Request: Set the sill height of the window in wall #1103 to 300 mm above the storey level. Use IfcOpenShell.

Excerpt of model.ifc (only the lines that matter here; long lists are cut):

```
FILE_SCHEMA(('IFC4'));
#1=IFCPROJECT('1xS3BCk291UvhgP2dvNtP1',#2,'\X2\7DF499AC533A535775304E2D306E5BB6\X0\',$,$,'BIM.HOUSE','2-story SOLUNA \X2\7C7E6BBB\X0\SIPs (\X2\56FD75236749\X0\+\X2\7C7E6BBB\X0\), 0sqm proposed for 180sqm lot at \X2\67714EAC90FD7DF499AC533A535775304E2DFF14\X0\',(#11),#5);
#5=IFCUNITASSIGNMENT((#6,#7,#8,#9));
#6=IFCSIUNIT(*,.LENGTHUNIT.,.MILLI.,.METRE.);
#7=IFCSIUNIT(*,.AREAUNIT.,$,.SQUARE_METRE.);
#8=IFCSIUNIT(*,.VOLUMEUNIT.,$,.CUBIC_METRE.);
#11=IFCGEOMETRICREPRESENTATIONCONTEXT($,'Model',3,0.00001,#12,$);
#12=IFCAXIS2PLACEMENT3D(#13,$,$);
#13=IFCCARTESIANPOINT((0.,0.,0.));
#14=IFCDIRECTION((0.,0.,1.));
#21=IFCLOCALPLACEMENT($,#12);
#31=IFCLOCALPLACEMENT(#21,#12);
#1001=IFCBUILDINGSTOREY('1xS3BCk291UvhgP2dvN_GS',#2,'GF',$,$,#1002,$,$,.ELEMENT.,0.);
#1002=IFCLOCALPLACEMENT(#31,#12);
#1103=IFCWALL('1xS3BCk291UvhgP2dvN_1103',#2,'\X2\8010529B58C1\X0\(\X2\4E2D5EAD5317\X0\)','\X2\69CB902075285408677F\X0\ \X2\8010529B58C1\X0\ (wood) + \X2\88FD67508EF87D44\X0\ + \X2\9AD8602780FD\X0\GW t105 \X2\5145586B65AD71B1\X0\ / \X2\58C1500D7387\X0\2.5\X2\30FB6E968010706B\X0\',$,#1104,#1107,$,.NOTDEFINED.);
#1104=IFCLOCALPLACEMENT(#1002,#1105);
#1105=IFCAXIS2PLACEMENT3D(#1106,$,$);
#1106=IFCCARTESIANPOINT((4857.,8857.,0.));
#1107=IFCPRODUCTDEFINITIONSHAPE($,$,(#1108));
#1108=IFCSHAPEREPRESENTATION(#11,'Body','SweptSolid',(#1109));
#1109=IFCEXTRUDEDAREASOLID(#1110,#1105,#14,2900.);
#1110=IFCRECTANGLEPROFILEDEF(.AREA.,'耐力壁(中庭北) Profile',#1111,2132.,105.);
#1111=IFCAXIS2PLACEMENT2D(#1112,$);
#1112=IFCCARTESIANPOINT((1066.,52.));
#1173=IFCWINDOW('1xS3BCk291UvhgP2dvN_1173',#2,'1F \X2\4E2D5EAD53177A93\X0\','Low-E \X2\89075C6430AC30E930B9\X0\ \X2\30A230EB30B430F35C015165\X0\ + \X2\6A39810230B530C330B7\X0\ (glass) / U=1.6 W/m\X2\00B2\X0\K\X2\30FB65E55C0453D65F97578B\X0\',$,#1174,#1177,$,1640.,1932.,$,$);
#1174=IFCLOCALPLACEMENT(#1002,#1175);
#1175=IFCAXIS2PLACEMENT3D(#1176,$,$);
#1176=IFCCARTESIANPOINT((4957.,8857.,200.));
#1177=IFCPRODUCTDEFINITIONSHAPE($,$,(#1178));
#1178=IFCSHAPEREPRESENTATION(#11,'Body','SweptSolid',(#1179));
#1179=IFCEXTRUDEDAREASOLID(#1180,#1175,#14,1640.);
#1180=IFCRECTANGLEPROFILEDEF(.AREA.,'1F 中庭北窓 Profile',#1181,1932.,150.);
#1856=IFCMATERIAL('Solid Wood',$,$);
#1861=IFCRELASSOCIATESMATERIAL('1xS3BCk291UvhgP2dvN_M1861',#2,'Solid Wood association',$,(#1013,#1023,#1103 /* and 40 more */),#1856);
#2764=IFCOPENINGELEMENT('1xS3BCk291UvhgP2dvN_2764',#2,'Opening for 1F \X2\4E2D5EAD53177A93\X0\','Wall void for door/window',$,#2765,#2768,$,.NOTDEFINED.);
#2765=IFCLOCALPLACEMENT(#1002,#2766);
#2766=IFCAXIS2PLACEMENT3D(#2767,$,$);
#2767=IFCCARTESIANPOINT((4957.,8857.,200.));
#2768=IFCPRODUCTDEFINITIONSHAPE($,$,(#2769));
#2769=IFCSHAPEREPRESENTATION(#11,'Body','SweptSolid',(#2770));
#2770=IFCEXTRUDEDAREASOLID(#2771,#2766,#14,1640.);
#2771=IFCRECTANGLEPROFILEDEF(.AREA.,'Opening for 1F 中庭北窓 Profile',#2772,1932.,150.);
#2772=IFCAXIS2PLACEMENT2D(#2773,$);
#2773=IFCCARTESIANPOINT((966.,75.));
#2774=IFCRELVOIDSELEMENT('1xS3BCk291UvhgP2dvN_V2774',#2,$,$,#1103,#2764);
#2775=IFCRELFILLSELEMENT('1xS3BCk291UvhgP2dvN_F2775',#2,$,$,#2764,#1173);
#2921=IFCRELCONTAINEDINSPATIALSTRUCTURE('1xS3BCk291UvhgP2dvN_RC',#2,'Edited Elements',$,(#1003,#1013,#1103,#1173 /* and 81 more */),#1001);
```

```python
import numpy as np
import ifcopenshell
import ifcopenshell.api.geometry
import ifcopenshell.geom
import ifcopenshell.util.element
import ifcopenshell.util.placement
import ifcopenshell.util.shape
import ifcopenshell.util.unit

model = ifcopenshell.open("model.ifc")
unit_scale = ifcopenshell.util.unit.calculate_unit_scale(model)

window = model.by_guid("1xS3BCk291UvhgP2dvN_1173")
opening = window.FillsVoids[0].RelatingOpeningElement
storey = ifcopenshell.util.element.get_container(window, ifc_class="IfcBuildingStorey")
level = ifcopenshell.util.placement.get_local_placement(storey.ObjectPlacement)[2, 3]

# The opening's origin need not be at the sill, so measure its lowest point.
shape = ifcopenshell.geom.create_shape(ifcopenshell.geom.settings(), opening)
bottom = ifcopenshell.util.shape.get_shape_bottom_elevation(shape, shape.geometry) / unit_scale
dz = level + 0.3 / unit_scale - bottom

shift = np.array([0.0, 0.0, dz])
# The window is not placed relative to its opening, so move both.
for product in (opening, window):
    matrix = ifcopenshell.util.placement.get_local_placement(product.ObjectPlacement)
    matrix[:3, 3] += shift
    ifcopenshell.api.geometry.edit_object_placement(model, product=product, matrix=matrix, is_si=False)

print(f"moved by {dz * unit_scale:+.3f} m")

model.write("model_v2.ifc")
```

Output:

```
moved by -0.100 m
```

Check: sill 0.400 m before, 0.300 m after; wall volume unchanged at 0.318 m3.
